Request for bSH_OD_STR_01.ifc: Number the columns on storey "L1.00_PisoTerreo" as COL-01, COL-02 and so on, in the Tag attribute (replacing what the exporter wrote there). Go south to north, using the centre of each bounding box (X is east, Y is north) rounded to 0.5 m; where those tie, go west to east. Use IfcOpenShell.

First a look at what the model holds.

```python
import ifcopenshell
import ifcopenshell.util.element
import ifcopenshell.util.placement

model = ifcopenshell.open("bSH_OD_STR_01.ifc")
print(model.schema)
storey = next(s for s in model.by_type("IfcBuildingStorey") if s.Name == "L1.00_PisoTerreo")
columns = [e for e in ifcopenshell.util.element.get_decomposition(storey) if e.is_a("IfcColumn")]
for e in sorted(columns, key=lambda e: e.id()):
    origin = ifcopenshell.util.placement.get_local_placement(e.ObjectPlacement)[:3, 3]
    print(e.id(), e.Tag, e.Name, origin.round(2) + 0.0, sep=" | ")
```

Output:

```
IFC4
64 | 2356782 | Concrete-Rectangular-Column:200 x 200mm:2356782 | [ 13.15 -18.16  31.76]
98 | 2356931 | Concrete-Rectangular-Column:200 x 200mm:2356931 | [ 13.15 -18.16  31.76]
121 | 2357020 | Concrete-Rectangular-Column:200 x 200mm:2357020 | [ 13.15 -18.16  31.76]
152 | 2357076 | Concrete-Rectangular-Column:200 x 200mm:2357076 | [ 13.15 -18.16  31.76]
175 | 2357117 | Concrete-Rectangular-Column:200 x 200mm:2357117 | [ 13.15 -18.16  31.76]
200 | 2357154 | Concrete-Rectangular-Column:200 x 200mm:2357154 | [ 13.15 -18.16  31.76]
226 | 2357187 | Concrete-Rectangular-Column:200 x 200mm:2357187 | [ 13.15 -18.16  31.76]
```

```python
import ifcopenshell
import ifcopenshell.geom
import ifcopenshell.util.element
import ifcopenshell.util.shape

model = ifcopenshell.open("bSH_OD_STR_01.ifc")
settings = ifcopenshell.geom.settings()
settings.set("use-world-coords", True)


def centre(element):
    shape = ifcopenshell.geom.create_shape(settings, element)
    return ifcopenshell.util.shape.get_bbox_centroid(shape.geometry)


storey = next(s for s in model.by_type("IfcBuildingStorey") if s.Name == "L1.00_PisoTerreo")
columns = [e for e in ifcopenshell.util.element.get_decomposition(storey) if e.is_a("IfcColumn")]

# Insertion points can sit at a corner or the storey origin, so sort by the geometry (in metres).
centres = {e: centre(e) for e in columns}
columns.sort(key=lambda e: (round(centres[e][1] / 0.5), centres[e][0]))

for i, e in enumerate(columns, start=1):
    number = f"COL-{i:02d}"
    e.Tag = number
    print(e.id(), number)

model.write("bSH_OD_STR_01_v2.ifc")
```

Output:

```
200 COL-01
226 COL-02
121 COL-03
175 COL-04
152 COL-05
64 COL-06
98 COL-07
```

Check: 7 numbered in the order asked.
